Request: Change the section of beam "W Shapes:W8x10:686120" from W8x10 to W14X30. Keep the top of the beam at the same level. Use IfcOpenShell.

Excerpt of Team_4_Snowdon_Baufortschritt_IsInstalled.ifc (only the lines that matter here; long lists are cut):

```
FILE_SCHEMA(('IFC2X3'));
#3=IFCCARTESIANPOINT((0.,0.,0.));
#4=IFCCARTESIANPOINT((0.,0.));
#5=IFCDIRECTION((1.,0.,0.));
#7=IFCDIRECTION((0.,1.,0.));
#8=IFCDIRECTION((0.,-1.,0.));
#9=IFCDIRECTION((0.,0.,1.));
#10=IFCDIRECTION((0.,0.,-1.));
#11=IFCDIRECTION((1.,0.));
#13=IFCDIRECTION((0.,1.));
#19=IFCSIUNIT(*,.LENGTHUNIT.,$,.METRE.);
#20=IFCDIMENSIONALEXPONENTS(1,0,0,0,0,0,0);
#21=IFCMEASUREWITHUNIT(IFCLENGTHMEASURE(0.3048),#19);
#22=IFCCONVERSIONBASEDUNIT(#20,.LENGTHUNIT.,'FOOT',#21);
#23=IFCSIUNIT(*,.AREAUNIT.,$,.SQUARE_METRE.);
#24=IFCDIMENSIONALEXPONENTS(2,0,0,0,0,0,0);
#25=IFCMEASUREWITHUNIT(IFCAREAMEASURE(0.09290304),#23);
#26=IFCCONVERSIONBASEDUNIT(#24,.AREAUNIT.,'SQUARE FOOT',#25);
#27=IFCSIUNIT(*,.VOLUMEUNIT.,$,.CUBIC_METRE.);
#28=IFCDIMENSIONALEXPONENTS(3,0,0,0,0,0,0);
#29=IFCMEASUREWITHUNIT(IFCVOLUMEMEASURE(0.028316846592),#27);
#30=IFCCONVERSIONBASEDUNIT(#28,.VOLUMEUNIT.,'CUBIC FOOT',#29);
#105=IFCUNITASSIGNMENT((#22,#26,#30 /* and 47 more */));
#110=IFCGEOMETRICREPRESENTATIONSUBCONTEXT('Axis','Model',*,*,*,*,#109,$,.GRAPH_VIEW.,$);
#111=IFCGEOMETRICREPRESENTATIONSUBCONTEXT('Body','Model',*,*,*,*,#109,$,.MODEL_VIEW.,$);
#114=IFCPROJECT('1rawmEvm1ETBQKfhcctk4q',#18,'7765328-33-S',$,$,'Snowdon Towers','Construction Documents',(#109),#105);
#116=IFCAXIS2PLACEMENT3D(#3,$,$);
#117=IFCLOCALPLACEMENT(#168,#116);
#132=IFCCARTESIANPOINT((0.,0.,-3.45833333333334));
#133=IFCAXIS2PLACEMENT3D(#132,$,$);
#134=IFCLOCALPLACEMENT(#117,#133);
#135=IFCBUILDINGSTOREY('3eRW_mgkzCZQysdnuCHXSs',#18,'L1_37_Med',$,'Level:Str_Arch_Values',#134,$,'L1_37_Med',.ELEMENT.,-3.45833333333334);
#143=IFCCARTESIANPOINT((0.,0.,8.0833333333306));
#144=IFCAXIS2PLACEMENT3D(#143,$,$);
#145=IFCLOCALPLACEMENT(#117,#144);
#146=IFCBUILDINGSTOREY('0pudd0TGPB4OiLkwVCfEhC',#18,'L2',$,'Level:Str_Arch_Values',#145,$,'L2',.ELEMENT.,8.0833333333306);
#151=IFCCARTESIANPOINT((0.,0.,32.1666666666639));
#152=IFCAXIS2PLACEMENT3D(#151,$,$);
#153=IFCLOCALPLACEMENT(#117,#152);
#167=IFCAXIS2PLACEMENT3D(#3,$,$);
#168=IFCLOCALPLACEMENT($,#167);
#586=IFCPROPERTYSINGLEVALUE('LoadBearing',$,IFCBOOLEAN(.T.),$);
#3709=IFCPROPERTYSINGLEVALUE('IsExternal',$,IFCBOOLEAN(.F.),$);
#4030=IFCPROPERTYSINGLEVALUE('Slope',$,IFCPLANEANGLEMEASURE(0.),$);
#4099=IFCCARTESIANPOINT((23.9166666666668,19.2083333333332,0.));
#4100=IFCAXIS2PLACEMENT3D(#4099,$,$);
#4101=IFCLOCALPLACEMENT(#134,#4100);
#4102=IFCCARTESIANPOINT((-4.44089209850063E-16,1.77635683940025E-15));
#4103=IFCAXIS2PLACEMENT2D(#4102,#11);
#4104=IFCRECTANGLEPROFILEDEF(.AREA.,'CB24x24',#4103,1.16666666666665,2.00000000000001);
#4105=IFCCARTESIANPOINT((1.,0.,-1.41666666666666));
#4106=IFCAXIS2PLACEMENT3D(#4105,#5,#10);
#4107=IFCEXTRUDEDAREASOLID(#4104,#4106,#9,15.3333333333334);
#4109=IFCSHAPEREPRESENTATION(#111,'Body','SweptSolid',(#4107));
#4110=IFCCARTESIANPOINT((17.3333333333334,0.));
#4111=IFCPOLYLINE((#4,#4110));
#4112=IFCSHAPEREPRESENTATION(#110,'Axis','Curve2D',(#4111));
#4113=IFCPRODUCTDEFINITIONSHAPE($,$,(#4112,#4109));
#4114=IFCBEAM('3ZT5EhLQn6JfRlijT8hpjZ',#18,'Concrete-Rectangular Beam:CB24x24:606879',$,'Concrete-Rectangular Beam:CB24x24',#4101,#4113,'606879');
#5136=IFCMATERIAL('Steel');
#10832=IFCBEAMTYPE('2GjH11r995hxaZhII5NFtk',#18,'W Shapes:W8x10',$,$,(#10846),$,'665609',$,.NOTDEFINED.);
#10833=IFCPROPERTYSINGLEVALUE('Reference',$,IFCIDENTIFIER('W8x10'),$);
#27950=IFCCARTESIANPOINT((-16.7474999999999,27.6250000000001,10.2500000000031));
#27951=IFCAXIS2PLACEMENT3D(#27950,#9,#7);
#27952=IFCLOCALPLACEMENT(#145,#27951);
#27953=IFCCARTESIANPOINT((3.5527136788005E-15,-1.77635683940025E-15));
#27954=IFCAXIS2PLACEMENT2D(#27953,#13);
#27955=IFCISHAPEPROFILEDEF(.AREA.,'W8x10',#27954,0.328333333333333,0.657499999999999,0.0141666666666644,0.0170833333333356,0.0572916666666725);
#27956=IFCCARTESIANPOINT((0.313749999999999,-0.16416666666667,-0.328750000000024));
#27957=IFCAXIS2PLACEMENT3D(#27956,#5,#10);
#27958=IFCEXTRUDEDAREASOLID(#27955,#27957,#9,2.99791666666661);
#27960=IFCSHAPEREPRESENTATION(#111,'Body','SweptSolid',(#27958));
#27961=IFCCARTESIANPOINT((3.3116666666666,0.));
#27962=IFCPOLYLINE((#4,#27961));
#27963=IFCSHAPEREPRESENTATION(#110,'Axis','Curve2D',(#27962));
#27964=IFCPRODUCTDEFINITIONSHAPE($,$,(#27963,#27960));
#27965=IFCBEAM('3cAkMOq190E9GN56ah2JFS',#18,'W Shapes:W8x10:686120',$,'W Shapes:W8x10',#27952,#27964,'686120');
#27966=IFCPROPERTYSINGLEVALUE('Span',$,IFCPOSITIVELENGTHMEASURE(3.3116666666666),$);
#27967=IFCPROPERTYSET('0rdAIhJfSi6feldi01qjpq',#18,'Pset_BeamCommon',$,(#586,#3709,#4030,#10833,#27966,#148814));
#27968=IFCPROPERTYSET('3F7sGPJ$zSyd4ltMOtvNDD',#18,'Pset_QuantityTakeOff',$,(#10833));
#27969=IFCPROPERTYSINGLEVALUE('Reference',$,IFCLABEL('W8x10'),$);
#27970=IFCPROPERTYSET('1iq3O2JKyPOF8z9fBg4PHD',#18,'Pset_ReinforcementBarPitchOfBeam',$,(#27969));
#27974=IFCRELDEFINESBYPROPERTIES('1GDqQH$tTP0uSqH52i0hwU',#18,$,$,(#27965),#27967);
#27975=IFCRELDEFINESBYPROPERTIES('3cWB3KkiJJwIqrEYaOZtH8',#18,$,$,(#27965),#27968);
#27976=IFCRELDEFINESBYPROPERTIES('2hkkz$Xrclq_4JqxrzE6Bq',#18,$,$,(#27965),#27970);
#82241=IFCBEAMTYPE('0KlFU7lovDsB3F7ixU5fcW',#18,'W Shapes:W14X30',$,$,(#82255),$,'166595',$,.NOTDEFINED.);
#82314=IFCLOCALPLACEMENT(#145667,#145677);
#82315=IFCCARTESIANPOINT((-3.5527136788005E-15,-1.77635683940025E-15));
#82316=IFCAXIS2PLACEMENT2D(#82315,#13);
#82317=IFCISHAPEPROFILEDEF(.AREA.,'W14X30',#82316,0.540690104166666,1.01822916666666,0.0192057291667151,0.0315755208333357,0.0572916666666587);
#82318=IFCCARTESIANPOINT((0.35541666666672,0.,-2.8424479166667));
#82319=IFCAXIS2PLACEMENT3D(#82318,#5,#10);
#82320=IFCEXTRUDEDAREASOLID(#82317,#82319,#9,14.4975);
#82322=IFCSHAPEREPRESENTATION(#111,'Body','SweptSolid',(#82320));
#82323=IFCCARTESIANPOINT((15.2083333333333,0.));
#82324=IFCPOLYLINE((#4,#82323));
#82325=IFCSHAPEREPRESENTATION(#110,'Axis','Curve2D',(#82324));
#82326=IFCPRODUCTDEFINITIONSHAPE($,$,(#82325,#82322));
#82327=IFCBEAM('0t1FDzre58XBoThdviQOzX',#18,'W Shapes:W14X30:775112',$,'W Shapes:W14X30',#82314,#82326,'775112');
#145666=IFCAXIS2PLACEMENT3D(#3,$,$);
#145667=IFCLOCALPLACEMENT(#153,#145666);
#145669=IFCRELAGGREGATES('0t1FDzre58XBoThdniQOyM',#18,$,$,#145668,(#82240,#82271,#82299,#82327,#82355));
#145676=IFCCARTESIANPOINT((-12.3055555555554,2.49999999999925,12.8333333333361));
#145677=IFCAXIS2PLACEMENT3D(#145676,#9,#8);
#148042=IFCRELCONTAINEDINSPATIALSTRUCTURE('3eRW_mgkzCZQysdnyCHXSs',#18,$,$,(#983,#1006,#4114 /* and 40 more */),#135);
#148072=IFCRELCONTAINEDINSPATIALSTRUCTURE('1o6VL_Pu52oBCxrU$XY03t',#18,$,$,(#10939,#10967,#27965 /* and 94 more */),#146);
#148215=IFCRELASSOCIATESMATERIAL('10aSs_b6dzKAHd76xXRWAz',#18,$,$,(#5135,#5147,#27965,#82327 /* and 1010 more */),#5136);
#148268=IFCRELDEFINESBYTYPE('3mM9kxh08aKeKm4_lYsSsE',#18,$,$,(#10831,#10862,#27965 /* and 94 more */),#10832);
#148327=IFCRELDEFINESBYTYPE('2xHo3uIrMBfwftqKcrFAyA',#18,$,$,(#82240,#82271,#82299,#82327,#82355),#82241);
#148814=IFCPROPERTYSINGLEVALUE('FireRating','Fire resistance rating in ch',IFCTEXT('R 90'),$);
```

```python
import ifcopenshell
import ifcopenshell.api.pset
import ifcopenshell.api.type
import ifcopenshell.util.element
import ifcopenshell.util.representation

model = ifcopenshell.open("Team_4_Snowdon_Baufortschritt_IsInstalled.ifc")

member = model.by_id(27965)
source = next(p for p in model.by_type("IfcIShapeProfileDef") if p.ProfileName == "W14X30")

body = ifcopenshell.util.representation.get_representation(member, "Model", "Body")
solid = body.Items[0]
old_profile = solid.SweptArea

# Copy the section's sizes but keep this member's own profile position.
profile = ifcopenshell.util.element.copy(model, source)
# Profiles are centred, so shift by half the change in depth to hold the top.
shift = (old_profile.OverallDepth - profile.OverallDepth) / 2
x, y = old_profile.Position.Location.Coordinates
up = (-1.0, 0.0)  # upwards, in the solid's own plane
location = model.createIfcCartesianPoint((x + up[0] * shift, y + up[1] * shift))
profile.Position = model.createIfcAxis2Placement2D(location, old_profile.Position.RefDirection)
solid.SweptArea = profile
if not model.get_total_inverses(old_profile):
    ifcopenshell.util.element.remove_deep2(model, old_profile)

new_type = model.by_guid("0KlFU7lovDsB3F7ixU5fcW")
ifcopenshell.api.type.assign_type(
    model, related_objects=[member], relating_type=new_type, should_map_representations=False
)
member.Name = member.Name.replace("W8x10", "W14X30")
member.ObjectType = "W Shapes:W14X30"
pset = model.by_id(ifcopenshell.util.element.get_pset(member, "Pset_BeamCommon", should_inherit=False)["id"])
ifcopenshell.api.pset.edit_pset(model, pset=pset, properties={"Reference": "W14X30"})
pset = model.by_id(ifcopenshell.util.element.get_pset(member, "Pset_QuantityTakeOff", should_inherit=False)["id"])
ifcopenshell.api.pset.edit_pset(model, pset=pset, properties={"Reference": "W14X30"})
pset = model.by_id(ifcopenshell.util.element.get_pset(member, "Pset_ReinforcementBarPitchOfBeam", should_inherit=False)["id"])
ifcopenshell.api.pset.edit_pset(model, pset=pset, properties={"Reference": "W14X30"})

print(solid.SweptArea)

model.write("Team_4_Snowdon_Baufortschritt_IsInstalled_updated.ifc")
```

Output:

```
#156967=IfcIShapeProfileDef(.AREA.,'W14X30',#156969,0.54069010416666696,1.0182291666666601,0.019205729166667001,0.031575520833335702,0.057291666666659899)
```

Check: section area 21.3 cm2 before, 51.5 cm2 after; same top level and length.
